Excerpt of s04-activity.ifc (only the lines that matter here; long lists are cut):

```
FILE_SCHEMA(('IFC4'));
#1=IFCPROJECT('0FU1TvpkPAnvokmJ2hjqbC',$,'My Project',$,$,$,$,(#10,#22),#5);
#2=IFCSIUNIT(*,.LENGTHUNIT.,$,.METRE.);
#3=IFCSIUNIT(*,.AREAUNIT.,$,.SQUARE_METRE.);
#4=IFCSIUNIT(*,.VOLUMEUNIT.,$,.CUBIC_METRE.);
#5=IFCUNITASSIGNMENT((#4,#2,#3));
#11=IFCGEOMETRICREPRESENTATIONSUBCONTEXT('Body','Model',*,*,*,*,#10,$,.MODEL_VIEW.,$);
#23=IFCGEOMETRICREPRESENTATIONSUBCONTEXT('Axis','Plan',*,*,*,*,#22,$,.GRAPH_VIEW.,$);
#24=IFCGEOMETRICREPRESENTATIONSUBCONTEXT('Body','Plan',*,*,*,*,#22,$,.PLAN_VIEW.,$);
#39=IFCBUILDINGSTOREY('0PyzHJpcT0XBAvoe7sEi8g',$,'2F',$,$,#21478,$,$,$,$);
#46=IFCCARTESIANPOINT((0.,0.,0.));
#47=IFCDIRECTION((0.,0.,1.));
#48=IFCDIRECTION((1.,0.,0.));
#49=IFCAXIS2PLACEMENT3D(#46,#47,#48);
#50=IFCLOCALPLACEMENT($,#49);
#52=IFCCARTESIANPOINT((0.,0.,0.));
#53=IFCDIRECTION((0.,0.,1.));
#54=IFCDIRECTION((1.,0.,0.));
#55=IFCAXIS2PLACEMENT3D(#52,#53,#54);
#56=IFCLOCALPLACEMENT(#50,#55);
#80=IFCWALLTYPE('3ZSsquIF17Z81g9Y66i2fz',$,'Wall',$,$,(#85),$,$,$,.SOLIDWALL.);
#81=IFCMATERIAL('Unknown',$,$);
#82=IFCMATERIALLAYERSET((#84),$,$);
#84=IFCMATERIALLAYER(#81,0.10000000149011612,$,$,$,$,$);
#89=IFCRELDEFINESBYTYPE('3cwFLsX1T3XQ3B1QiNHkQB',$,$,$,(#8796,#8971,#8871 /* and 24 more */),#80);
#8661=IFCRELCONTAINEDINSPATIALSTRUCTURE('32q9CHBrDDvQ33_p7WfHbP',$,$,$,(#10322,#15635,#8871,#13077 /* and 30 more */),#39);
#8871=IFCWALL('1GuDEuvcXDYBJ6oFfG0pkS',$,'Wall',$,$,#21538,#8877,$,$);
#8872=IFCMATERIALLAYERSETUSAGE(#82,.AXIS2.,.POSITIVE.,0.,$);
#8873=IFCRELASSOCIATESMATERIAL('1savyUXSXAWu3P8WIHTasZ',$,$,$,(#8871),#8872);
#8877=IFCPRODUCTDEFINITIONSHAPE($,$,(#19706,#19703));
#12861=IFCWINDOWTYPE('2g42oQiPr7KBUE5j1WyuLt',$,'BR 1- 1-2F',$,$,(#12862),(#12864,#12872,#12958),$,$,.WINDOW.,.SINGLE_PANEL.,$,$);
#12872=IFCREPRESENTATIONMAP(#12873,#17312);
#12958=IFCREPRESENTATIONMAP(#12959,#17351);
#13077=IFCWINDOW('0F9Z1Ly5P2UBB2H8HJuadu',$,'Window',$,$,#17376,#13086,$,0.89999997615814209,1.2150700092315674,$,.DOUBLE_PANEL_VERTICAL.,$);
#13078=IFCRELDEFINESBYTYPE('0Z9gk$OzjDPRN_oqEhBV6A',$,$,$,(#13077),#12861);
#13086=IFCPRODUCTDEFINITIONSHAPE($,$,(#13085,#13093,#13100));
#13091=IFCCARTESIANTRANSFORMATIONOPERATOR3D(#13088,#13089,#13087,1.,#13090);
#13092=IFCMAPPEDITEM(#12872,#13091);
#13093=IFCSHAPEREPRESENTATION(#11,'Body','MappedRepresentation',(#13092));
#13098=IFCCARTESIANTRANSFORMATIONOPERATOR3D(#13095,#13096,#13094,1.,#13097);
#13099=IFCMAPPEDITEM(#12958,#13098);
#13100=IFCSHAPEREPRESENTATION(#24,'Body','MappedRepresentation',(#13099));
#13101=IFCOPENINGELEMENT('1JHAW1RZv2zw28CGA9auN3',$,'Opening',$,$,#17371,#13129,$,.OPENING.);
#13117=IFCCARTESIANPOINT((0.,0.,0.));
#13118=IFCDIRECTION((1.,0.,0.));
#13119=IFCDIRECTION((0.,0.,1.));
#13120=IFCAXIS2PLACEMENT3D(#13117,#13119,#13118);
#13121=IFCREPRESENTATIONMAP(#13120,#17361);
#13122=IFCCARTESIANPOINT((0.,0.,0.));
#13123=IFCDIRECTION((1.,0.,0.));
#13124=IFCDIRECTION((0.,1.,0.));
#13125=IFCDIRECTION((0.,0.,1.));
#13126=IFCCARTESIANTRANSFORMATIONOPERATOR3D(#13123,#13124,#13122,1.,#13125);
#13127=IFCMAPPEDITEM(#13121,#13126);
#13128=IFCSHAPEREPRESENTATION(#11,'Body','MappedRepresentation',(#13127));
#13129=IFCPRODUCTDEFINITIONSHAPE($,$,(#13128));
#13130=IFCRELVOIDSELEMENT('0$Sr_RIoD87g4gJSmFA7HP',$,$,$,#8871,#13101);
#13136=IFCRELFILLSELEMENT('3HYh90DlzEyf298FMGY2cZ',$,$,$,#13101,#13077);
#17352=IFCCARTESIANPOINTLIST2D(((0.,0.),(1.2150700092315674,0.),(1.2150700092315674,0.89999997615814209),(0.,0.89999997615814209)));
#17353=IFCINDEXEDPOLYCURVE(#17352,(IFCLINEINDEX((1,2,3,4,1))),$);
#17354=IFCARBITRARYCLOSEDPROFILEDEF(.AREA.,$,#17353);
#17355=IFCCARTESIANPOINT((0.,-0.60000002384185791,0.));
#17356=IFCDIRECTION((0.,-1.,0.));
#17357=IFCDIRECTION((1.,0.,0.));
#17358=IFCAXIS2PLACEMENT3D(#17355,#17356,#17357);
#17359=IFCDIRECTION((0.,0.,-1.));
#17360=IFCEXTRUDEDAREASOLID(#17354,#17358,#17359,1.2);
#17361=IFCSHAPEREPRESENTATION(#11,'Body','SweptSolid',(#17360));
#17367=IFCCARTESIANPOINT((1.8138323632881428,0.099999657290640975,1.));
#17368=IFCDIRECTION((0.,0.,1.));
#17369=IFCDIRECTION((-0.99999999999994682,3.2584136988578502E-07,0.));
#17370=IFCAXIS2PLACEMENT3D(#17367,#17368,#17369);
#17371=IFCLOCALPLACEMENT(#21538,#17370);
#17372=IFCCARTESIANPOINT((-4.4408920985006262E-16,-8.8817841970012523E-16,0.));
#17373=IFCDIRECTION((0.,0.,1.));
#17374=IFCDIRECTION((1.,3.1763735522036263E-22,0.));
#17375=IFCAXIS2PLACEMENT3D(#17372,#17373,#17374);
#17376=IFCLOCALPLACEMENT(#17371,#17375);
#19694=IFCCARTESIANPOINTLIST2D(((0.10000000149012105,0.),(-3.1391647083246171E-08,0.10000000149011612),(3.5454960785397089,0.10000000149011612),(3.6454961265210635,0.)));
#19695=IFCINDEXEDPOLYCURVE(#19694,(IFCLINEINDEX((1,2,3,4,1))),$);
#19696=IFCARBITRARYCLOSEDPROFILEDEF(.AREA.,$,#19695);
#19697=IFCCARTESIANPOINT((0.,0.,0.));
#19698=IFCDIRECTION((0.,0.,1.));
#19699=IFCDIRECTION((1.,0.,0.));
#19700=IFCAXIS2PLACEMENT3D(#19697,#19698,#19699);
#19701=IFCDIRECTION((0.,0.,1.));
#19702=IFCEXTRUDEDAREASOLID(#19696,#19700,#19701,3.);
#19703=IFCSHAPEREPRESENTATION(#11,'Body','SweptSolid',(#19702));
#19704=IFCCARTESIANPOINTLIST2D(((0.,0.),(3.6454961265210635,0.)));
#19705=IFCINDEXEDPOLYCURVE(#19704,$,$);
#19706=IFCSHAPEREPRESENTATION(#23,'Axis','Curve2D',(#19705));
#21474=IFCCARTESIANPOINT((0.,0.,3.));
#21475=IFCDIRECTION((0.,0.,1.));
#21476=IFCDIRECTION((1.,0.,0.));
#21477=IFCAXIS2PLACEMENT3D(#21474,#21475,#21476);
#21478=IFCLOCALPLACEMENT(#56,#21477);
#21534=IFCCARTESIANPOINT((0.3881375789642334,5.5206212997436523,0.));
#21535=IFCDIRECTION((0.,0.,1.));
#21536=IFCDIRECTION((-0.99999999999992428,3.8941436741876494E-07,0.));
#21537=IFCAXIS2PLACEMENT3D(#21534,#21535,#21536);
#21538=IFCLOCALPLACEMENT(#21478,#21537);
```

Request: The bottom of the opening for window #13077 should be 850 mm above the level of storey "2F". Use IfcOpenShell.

```python
import numpy as np
import ifcopenshell
import ifcopenshell.api.geometry
import ifcopenshell.geom
import ifcopenshell.util.element
import ifcopenshell.util.placement
import ifcopenshell.util.shape
import ifcopenshell.util.unit

model = ifcopenshell.open("s04-activity.ifc")
unit_scale = ifcopenshell.util.unit.calculate_unit_scale(model)

window = model.by_guid("0F9Z1Ly5P2UBB2H8HJuadu")
opening = window.FillsVoids[0].RelatingOpeningElement
storey = ifcopenshell.util.element.get_container(window, ifc_class="IfcBuildingStorey")
level = ifcopenshell.util.placement.get_local_placement(storey.ObjectPlacement)[2, 3]

# The opening's origin need not be at the sill, so measure its lowest point.
shape = ifcopenshell.geom.create_shape(ifcopenshell.geom.settings(), opening)
bottom = ifcopenshell.util.shape.get_shape_bottom_elevation(shape, shape.geometry) / unit_scale
dz = level + 0.85 / unit_scale - bottom

shift = np.array([0.0, 0.0, dz])
# The window is placed relative to its opening, so it follows when the opening moves.
matrix = ifcopenshell.util.placement.get_local_placement(opening.ObjectPlacement)
matrix[:3, 3] += shift
ifcopenshell.api.geometry.edit_object_placement(
    model, product=opening, matrix=matrix, is_si=False, should_transform_children=True
)

print(f"moved by {dz * unit_scale:+.3f} m")

model.write("s04-activity_rev.ifc")
```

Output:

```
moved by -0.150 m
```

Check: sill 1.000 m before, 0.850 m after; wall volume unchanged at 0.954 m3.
